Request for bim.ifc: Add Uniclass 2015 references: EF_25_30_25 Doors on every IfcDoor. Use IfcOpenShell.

First a look at what the model holds.

```python
import ifcopenshell

model = ifcopenshell.open("bim.ifc")
print(model.schema)
print("classifications:", [c.Name for c in model.by_type("IfcClassification")])
for ifc_class in ("IfcDoor", "IfcRoof", "IfcStair", "IfcWall", "IfcWindow"):
    print(ifc_class, len(model.by_type(ifc_class)))
```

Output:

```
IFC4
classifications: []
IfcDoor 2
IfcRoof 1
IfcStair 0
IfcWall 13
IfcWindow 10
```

```python
import ifcopenshell
import ifcopenshell.api.classification

model = ifcopenshell.open("bim.ifc")

system = ifcopenshell.api.classification.add_classification(model, classification="Uniclass 2015")

codes = {
    "IfcDoor": ("EF_25_30_25", "Doors"),
}
for ifc_class, (code, name) in codes.items():
    products = model.by_type(ifc_class)
    ifcopenshell.api.classification.add_reference(
        model, products=products, classification=system, identification=code, name=name
    )
    print(code, len(products))

model.write("bim_v2.ifc")
```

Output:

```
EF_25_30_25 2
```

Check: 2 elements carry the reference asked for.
